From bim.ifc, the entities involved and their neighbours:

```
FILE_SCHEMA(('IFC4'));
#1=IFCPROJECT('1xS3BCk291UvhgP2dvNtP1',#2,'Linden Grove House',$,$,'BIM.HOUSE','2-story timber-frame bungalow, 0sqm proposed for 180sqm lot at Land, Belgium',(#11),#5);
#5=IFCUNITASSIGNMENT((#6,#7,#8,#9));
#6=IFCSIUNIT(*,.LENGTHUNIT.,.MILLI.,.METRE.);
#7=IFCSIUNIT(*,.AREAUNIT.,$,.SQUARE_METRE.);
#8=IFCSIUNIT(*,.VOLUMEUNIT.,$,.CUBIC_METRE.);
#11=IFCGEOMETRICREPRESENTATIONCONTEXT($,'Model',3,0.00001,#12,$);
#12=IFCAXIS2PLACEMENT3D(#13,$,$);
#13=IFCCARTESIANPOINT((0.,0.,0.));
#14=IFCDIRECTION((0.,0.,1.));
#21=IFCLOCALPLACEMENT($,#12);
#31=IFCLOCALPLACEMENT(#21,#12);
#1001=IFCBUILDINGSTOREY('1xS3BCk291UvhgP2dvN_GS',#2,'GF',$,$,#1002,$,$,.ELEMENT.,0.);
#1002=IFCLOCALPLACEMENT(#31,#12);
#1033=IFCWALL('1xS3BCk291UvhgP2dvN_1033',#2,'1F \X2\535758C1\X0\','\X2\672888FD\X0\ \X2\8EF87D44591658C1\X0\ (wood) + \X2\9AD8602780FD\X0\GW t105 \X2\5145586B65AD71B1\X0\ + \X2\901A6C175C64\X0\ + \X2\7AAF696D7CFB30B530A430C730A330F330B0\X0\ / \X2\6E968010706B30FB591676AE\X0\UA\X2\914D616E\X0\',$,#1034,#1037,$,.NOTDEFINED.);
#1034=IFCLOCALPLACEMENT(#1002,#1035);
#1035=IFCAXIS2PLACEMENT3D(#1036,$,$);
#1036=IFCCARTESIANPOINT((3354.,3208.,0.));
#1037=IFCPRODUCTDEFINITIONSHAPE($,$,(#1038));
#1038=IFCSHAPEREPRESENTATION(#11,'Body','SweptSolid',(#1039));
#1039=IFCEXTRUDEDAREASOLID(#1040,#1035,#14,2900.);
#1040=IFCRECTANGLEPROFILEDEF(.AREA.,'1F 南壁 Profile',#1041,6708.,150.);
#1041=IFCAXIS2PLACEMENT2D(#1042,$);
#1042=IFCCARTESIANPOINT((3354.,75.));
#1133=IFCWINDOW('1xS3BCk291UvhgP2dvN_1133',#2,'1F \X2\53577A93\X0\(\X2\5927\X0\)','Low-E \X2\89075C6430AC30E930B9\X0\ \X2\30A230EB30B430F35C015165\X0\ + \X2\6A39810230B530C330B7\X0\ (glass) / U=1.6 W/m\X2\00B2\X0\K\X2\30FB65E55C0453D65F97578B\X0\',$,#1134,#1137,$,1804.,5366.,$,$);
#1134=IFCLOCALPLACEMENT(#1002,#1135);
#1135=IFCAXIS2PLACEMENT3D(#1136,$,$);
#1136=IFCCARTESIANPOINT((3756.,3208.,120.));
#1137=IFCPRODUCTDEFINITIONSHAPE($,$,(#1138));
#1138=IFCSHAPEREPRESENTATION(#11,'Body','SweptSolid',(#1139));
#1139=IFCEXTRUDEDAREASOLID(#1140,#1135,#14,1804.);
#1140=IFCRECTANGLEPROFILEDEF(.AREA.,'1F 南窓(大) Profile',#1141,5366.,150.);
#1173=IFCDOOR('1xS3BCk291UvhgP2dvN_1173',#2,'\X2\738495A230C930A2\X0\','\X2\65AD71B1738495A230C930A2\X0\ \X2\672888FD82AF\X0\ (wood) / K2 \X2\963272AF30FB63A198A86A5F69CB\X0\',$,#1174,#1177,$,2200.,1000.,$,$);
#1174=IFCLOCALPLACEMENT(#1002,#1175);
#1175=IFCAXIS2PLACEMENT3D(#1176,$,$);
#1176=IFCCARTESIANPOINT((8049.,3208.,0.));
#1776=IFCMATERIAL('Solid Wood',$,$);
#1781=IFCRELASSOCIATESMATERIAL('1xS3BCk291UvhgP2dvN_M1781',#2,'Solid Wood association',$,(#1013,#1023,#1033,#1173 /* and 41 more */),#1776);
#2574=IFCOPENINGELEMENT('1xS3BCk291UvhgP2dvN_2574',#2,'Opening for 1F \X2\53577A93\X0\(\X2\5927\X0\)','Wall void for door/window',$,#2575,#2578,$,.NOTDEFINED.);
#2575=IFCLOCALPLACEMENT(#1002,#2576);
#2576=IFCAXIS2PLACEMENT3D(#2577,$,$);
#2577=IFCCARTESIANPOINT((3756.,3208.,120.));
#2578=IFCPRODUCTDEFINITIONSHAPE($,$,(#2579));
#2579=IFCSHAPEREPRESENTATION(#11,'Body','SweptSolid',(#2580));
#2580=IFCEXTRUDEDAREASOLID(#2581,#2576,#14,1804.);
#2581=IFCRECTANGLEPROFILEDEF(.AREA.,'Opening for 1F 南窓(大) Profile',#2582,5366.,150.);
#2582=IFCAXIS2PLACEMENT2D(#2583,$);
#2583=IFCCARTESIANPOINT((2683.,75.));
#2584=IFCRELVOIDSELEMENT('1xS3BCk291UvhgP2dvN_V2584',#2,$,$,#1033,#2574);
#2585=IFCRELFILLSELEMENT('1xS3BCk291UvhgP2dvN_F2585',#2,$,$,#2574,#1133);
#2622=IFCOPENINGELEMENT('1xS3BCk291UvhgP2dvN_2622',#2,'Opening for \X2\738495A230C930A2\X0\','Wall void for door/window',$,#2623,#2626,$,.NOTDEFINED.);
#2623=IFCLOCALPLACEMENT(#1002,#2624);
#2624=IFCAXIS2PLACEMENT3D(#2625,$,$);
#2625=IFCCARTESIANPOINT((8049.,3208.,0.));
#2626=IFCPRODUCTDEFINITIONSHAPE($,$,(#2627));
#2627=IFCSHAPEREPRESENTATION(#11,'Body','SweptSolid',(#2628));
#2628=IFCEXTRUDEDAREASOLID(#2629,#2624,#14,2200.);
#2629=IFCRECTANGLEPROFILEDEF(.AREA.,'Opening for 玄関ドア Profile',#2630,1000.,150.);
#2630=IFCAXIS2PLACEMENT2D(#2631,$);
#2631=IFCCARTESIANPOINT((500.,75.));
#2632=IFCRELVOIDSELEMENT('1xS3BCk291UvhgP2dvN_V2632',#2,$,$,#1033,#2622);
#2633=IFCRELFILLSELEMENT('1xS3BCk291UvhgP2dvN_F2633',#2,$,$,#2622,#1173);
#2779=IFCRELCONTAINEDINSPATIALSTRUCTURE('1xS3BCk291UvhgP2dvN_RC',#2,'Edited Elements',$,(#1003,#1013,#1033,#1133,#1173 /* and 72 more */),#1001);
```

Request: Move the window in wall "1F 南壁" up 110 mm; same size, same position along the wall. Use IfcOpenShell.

```python
import numpy as np
import ifcopenshell
import ifcopenshell.api.geometry
import ifcopenshell.util.placement
import ifcopenshell.util.unit

model = ifcopenshell.open("bim.ifc")
unit_scale = ifcopenshell.util.unit.calculate_unit_scale(model)

window = model.by_id(1133)
opening = window.FillsVoids[0].RelatingOpeningElement
dz = 110.0

shift = np.array([0.0, 0.0, dz])
# The window is not placed relative to its opening, so move both.
for product in (opening, window):
    matrix = ifcopenshell.util.placement.get_local_placement(product.ObjectPlacement)
    matrix[:3, 3] += shift
    ifcopenshell.api.geometry.edit_object_placement(model, product=product, matrix=matrix, is_si=False)

print(f"moved by {dz * unit_scale:+.3f} m")

model.write("bim_rev.ifc")
```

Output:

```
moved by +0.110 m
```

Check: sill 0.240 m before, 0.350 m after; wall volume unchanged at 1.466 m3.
